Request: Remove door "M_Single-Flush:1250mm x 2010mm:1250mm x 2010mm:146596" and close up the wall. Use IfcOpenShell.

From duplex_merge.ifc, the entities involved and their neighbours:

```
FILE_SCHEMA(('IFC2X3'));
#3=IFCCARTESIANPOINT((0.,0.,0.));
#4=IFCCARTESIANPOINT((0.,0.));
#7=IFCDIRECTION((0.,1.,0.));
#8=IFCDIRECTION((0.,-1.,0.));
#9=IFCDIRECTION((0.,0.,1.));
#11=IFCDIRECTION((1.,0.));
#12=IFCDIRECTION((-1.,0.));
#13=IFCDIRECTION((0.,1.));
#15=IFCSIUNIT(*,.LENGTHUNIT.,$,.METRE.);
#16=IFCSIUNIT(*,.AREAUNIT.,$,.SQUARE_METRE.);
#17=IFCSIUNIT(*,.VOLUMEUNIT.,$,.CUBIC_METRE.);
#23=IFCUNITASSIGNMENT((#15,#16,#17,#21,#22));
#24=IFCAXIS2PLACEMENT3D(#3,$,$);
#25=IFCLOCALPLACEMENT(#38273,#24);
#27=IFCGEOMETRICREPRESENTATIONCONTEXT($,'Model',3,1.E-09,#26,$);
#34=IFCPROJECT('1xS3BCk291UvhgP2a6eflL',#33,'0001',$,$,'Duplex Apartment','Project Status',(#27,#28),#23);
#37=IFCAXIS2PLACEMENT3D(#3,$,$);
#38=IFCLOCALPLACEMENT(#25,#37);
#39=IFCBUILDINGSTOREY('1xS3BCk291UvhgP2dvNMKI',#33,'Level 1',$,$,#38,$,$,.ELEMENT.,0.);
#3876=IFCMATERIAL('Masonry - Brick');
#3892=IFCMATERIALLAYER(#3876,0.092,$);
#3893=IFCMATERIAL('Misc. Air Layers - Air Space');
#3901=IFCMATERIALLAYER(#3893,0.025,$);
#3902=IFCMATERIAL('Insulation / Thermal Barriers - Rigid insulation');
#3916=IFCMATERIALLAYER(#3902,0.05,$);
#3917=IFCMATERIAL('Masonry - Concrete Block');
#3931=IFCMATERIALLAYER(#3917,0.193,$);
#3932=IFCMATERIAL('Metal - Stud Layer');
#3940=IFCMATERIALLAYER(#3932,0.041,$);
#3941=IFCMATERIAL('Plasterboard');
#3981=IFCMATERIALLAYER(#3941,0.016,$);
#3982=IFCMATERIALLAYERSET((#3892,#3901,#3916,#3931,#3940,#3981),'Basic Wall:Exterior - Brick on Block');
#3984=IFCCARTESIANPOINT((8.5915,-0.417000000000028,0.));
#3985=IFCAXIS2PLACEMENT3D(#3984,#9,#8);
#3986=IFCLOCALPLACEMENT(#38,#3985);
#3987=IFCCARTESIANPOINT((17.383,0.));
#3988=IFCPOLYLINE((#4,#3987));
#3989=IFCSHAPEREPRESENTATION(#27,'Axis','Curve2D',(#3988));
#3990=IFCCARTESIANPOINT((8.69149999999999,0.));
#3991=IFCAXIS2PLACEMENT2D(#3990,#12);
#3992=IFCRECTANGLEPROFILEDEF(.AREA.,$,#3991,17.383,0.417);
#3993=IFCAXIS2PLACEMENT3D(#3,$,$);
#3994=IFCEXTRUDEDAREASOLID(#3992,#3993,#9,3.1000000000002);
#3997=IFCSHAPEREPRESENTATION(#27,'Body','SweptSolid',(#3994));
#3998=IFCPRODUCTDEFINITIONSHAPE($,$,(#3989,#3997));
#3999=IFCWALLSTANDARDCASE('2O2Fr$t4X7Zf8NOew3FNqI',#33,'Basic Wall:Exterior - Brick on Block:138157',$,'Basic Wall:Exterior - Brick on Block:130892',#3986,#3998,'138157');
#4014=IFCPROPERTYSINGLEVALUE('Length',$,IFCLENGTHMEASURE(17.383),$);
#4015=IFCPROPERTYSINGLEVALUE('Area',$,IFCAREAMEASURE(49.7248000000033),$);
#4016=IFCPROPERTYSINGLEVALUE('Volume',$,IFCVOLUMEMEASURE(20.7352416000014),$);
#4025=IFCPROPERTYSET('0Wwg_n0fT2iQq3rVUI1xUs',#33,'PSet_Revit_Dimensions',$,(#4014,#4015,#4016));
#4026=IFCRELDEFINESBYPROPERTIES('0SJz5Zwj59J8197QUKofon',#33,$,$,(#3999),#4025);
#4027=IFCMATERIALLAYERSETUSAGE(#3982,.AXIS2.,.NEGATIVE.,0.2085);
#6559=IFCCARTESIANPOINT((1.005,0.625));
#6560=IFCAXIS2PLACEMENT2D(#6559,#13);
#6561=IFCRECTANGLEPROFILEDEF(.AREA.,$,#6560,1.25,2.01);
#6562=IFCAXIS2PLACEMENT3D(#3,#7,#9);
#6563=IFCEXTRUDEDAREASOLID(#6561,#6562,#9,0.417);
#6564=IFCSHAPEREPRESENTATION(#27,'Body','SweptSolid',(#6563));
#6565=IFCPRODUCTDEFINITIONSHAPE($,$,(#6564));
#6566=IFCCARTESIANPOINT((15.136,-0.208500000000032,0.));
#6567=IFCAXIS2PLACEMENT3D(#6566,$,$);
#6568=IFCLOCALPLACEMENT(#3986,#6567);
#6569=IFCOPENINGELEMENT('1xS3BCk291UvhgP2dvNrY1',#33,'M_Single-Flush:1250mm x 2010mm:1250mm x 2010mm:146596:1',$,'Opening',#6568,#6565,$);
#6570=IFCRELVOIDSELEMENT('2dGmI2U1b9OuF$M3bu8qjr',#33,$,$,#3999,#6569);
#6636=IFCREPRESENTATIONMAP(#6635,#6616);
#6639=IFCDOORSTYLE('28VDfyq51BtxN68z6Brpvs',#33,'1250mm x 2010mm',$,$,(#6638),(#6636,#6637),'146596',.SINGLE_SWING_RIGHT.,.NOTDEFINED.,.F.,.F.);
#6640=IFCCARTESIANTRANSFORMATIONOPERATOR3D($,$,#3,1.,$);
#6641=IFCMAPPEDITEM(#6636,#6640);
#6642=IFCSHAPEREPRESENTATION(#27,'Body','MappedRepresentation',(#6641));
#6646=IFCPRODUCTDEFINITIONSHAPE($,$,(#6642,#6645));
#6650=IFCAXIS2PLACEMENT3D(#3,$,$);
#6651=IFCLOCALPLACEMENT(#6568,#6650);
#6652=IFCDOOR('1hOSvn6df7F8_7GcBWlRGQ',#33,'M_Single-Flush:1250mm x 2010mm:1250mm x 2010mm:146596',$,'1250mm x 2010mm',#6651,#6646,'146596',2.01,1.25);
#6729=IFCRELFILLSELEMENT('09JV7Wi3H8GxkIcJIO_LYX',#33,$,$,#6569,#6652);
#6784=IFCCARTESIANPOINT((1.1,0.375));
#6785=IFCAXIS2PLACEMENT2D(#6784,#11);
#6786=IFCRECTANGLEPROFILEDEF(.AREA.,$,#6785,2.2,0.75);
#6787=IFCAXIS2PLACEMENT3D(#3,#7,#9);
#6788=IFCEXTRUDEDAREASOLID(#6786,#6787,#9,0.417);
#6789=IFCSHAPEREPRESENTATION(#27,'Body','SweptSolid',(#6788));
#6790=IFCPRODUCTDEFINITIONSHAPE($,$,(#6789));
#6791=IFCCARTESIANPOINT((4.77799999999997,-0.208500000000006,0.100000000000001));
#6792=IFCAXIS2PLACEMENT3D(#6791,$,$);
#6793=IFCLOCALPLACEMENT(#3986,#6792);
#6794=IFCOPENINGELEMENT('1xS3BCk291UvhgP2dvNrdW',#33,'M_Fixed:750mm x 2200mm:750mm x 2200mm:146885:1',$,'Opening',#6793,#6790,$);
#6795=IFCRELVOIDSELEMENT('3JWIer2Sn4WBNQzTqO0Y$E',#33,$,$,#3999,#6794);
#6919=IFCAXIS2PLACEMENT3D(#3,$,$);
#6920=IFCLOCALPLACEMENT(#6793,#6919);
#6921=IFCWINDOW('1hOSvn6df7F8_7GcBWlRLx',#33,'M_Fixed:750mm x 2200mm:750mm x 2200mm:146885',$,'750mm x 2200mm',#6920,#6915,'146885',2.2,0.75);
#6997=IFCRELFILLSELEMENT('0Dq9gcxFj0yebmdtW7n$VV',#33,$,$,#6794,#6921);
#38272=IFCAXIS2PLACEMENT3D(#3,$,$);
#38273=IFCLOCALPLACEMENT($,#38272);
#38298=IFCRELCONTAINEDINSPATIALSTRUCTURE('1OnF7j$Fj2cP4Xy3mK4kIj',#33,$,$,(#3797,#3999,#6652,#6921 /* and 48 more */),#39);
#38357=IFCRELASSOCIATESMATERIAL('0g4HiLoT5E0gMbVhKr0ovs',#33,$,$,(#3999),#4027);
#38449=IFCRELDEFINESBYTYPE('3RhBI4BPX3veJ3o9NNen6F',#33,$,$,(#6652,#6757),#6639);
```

```python
import ifcopenshell
import ifcopenshell.api.feature
import ifcopenshell.api.pset
import ifcopenshell.api.root
import ifcopenshell.geom
import ifcopenshell.util.element
import ifcopenshell.util.shape
import ifcopenshell.util.unit

model = ifcopenshell.open("duplex_merge.ifc")
area_scale = ifcopenshell.util.unit.calculate_unit_scale(model, "AREAUNIT")
volume_scale = ifcopenshell.util.unit.calculate_unit_scale(model, "VOLUMEUNIT")
settings = ifcopenshell.geom.settings()


def volume(element):
    """Net volume in cubic metres, openings subtracted."""
    shape = ifcopenshell.geom.create_shape(settings, element)
    return ifcopenshell.util.shape.get_volume(shape.geometry)


door = model.by_guid("1hOSvn6df7F8_7GcBWlRGQ")
opening = door.FillsVoids[0].RelatingOpeningElement
wall = opening.VoidsElements[0].RelatingBuildingElement
before = volume(wall)

ifcopenshell.api.root.remove_product(model, product=door)
ifcopenshell.api.feature.remove_feature(model, feature=opening)

after = volume(wall)
thickness = 0.417  # wall thickness in metres

# Update the wall's stored quantities.
pset = model.by_id(ifcopenshell.util.element.get_pset(wall, "PSet_Revit_Dimensions", should_inherit=False)["id"])
ifcopenshell.api.pset.edit_pset(model, pset=pset, properties={
    "Area": model.create_entity("IfcAreaMeasure", after / thickness / area_scale),
    "Volume": model.create_entity("IfcVolumeMeasure", after / volume_scale),
})

print(f"wall volume {before:.3f} -> {after:.3f} m3")

model.write("duplex_merge-out.ifc")
```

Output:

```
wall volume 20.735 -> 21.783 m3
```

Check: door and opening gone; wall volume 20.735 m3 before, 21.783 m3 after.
